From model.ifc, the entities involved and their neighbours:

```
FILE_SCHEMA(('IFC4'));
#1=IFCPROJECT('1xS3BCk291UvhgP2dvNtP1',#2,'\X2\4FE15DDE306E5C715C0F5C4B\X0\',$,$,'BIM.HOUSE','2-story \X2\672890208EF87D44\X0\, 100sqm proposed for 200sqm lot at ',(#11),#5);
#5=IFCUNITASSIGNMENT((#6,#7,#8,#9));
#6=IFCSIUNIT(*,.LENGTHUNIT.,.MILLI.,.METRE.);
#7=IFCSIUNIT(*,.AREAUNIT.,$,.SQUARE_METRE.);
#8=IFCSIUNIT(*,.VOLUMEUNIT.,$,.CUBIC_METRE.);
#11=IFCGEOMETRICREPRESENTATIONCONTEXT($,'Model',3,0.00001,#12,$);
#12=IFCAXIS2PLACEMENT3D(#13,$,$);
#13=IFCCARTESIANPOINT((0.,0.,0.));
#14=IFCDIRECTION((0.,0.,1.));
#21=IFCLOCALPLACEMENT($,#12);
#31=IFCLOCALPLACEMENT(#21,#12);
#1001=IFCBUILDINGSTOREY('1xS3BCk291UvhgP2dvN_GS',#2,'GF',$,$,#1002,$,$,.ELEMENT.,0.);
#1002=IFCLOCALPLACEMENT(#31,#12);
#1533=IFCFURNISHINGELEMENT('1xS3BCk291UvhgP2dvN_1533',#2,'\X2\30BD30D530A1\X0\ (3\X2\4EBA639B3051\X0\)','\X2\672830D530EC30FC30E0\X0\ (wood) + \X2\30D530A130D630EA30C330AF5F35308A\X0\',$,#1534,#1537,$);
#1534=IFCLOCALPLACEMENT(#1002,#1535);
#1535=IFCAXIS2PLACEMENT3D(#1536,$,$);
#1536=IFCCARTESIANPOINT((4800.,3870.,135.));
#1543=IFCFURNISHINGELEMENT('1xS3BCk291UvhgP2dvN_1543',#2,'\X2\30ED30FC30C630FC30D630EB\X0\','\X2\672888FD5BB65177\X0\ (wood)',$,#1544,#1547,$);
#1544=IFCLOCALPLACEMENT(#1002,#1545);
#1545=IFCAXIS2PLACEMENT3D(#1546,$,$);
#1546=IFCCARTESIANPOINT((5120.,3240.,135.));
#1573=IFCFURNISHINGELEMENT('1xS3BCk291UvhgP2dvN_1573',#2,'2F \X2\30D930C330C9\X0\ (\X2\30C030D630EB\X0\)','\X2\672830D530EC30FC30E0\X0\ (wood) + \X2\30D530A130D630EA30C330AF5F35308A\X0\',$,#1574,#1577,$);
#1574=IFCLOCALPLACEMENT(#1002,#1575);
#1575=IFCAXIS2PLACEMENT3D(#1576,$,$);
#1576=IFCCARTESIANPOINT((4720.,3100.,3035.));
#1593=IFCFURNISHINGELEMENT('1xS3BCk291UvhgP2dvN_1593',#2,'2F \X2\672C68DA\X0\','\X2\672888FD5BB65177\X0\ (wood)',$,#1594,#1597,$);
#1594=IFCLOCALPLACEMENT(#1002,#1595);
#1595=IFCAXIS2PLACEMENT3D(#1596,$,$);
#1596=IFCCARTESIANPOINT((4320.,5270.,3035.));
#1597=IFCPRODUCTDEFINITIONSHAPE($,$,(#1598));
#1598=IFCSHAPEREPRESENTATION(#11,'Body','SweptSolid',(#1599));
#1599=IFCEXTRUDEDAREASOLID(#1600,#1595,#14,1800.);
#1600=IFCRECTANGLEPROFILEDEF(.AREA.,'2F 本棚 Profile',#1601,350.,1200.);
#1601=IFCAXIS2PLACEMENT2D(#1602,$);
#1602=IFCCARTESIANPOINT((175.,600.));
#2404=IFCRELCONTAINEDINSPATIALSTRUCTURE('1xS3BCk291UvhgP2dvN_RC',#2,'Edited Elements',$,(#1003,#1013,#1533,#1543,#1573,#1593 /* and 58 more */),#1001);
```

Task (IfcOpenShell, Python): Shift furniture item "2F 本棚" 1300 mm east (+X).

```python
import ifcopenshell
import ifcopenshell.api.geometry
import ifcopenshell.util.placement

model = ifcopenshell.open("model.ifc")

item = model.by_guid("1xS3BCk291UvhgP2dvN_1593")
matrix = ifcopenshell.util.placement.get_local_placement(item.ObjectPlacement)
matrix[0, 3] += 1300.0
ifcopenshell.api.geometry.edit_object_placement(model, product=item, matrix=matrix, is_si=False)

print(ifcopenshell.util.placement.get_local_placement(item.ObjectPlacement).round(3) + 0.0)

model.write("model_rev.ifc")
```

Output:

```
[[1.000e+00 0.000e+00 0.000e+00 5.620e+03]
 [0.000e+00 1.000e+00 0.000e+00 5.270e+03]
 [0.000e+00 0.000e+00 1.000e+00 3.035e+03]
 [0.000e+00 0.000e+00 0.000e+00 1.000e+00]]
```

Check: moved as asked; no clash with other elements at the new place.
